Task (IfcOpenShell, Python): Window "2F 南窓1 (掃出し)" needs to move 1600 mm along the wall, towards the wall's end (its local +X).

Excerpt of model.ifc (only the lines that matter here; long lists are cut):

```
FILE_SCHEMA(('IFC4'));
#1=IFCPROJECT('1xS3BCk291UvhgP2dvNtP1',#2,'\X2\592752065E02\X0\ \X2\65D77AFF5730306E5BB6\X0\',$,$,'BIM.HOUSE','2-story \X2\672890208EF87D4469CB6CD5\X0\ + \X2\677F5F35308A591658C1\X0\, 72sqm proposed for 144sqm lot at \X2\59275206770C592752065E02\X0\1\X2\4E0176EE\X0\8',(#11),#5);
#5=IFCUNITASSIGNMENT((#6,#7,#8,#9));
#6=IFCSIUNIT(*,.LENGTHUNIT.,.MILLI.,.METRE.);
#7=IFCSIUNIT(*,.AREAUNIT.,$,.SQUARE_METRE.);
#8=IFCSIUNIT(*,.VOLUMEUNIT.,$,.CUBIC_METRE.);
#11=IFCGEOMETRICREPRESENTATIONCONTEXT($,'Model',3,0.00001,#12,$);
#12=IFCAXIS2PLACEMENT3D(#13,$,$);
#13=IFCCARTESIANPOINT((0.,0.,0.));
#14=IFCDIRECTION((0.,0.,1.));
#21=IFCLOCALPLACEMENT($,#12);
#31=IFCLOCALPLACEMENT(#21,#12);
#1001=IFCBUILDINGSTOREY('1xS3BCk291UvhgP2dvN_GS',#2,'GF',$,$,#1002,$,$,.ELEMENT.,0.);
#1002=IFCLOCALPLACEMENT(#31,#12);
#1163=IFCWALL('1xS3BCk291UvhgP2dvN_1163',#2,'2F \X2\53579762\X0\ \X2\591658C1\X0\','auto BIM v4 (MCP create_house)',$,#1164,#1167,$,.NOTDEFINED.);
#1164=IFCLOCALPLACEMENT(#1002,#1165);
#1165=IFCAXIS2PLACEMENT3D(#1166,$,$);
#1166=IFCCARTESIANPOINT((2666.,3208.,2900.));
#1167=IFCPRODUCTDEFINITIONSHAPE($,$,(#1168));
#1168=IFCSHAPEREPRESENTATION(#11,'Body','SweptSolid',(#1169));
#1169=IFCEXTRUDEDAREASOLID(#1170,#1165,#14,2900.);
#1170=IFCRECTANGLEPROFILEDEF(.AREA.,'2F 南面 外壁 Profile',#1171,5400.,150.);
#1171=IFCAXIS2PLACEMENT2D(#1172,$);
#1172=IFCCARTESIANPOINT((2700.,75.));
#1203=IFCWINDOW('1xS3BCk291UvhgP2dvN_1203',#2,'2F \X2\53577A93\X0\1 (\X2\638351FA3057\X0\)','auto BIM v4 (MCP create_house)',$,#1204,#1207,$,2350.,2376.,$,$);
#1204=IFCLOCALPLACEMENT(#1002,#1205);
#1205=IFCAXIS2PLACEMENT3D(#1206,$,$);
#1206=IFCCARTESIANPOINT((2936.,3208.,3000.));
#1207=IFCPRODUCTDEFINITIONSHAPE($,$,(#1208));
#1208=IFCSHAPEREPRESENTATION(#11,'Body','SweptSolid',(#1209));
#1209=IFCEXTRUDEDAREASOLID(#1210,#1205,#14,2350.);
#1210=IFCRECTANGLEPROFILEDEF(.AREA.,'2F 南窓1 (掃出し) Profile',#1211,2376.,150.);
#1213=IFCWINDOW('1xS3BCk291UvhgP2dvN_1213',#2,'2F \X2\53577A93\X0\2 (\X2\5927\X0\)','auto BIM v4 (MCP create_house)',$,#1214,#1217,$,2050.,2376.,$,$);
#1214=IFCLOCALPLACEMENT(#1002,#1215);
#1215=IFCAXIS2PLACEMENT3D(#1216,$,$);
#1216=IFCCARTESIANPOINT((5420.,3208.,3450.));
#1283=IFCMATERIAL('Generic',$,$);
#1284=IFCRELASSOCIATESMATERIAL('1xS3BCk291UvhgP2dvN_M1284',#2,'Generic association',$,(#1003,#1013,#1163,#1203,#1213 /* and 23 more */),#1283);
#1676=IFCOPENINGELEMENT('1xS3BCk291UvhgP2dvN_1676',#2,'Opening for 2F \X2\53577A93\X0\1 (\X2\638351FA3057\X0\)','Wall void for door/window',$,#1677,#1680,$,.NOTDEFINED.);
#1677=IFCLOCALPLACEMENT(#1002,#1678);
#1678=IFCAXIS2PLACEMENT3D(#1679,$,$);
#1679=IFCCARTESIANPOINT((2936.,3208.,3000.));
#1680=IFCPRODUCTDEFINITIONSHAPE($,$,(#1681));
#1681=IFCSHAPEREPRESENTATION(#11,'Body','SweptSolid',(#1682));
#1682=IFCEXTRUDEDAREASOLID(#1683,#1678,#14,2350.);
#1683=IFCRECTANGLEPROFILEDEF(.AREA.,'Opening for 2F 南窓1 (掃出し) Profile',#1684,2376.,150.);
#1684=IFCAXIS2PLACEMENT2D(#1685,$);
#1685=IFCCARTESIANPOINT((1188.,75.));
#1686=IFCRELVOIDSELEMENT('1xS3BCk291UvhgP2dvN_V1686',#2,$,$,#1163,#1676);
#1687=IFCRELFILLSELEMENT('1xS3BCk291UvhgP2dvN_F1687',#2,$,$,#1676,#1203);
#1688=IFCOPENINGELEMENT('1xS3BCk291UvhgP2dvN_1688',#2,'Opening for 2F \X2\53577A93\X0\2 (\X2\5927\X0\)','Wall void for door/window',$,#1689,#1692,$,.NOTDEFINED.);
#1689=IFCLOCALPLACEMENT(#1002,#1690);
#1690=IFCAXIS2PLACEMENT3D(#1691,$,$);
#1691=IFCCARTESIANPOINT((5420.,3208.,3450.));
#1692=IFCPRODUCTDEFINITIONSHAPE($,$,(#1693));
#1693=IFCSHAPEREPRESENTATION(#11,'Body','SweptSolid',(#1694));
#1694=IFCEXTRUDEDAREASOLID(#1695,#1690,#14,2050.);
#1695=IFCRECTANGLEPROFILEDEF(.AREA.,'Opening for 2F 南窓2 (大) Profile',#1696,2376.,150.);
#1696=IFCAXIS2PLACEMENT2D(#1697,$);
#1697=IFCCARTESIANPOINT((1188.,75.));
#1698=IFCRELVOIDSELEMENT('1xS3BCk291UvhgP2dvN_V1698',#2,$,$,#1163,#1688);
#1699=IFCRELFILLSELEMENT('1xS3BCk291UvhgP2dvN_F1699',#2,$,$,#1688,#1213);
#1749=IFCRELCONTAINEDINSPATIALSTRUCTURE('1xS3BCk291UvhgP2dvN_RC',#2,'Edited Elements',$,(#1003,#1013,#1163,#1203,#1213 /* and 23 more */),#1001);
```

```python
import ifcopenshell
import ifcopenshell.api.geometry
import ifcopenshell.util.placement
import ifcopenshell.util.unit

model = ifcopenshell.open("model.ifc")
unit_scale = ifcopenshell.util.unit.calculate_unit_scale(model)

window = model.by_guid("1xS3BCk291UvhgP2dvN_1203")
opening = window.FillsVoids[0].RelatingOpeningElement
wall = opening.VoidsElements[0].RelatingBuildingElement

wall_matrix = ifcopenshell.util.placement.get_local_placement(wall.ObjectPlacement)
shift = wall_matrix[:3, 0] * 1.6 / unit_scale
before = ifcopenshell.util.placement.get_local_placement(window.ObjectPlacement)[:3, 3].copy()

# The window is not placed relative to its opening, so move both.
for product in (opening, window):
    matrix = ifcopenshell.util.placement.get_local_placement(product.ObjectPlacement)
    matrix[:3, 3] += shift
    ifcopenshell.api.geometry.edit_object_placement(model, product=product, matrix=matrix, is_si=False)

after = ifcopenshell.util.placement.get_local_placement(window.ObjectPlacement)[:3, 3]
print("window moved by", (after - before).round(3) + 0.0)

model.write("model_v2.ifc")
```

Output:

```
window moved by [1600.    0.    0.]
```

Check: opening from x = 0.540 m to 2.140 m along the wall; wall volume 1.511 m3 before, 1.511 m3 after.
